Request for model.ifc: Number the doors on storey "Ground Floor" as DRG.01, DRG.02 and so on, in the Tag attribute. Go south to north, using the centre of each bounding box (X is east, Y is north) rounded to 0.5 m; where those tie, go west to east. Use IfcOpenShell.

First a look at what the model holds.

```python
import ifcopenshell
import ifcopenshell.util.element
import ifcopenshell.util.placement

model = ifcopenshell.open("model.ifc")
print(model.schema)
storey = next(s for s in model.by_type("IfcBuildingStorey") if s.Name == "Ground Floor")
doors = [e for e in ifcopenshell.util.element.get_decomposition(storey) if e.is_a("IfcDoor")]
for e in sorted(doors, key=lambda e: e.id()):
    origin = ifcopenshell.util.placement.get_local_placement(e.ObjectPlacement)[:3, 3]
    print(e.id(), e.Tag, e.Name, origin.round(2) + 0.0, sep=" | ")
```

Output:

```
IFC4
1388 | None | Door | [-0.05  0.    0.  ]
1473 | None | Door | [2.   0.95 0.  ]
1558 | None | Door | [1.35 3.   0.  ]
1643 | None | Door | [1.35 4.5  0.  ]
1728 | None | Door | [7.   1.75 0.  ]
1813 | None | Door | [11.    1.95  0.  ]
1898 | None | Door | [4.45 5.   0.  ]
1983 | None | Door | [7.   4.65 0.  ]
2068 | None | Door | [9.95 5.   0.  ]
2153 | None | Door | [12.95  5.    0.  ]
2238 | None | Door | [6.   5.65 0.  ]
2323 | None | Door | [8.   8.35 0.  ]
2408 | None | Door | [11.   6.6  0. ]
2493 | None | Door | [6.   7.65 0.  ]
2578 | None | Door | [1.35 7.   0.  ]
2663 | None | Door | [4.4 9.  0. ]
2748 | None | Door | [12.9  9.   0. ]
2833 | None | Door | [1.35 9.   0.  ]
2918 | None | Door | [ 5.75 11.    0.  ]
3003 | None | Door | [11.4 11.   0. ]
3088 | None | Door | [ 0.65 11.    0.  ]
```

```python
import ifcopenshell
import ifcopenshell.geom
import ifcopenshell.util.element
import ifcopenshell.util.shape

model = ifcopenshell.open("model.ifc")
settings = ifcopenshell.geom.settings()
settings.set("use-world-coords", True)


def centre(element):
    shape = ifcopenshell.geom.create_shape(settings, element)
    return ifcopenshell.util.shape.get_bbox_centroid(shape.geometry)


storey = next(s for s in model.by_type("IfcBuildingStorey") if s.Name == "Ground Floor")
doors = [e for e in ifcopenshell.util.element.get_decomposition(storey) if e.is_a("IfcDoor")]

# Insertion points can sit at a corner or the storey origin, so sort by the geometry (in metres).
centres = {e: centre(e) for e in doors}
doors.sort(key=lambda e: (round(centres[e][1] / 0.5), centres[e][0]))

for i, e in enumerate(doors, start=1):
    number = f"DRG.{i:02d}"
    e.Tag = number
    print(e.id(), number)

model.write("model_edited.ifc")
```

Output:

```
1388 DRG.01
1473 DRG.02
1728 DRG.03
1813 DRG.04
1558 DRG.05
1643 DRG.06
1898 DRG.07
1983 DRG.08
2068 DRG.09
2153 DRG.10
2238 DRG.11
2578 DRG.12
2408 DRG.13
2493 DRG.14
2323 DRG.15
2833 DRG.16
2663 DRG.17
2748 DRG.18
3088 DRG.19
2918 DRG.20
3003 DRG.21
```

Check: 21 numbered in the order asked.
